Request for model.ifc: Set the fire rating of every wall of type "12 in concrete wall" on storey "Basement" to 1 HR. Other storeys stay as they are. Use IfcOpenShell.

First a look at what the model holds.

```python
import ifcopenshell
import ifcopenshell.util.element

model = ifcopenshell.open("model.ifc")
print(model.schema)
storey = next(s for s in model.by_type("IfcBuildingStorey") if s.Name == "Basement")
walls = [e for e in ifcopenshell.util.element.get_decomposition(storey) if e.is_a("IfcWall")]
seen = {}
for e in walls:
    element_type = ifcopenshell.util.element.get_type(e)
    key = (element_type.Name if element_type != e and element_type else None, ifcopenshell.util.element.get_pset(e, "Pset_WallCommon", "FireRating"))
    seen[key] = seen.get(key, 0) + 1
for (name, value), count in sorted(seen.items(), key=str):
    print(count, "x", name, "|", value)
```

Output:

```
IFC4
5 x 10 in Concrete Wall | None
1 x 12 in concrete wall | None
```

```python
import ifcopenshell
import ifcopenshell.api.pset
import ifcopenshell.util.element

model = ifcopenshell.open("model.ifc")

storey = next(s for s in model.by_type("IfcBuildingStorey") if s.Name == "Basement")
walls = [e for e in ifcopenshell.util.element.get_decomposition(storey) if e.is_a("IfcWall")]

count = 0
for e in walls:
    element_type = ifcopenshell.util.element.get_type(e)
    if element_type in (None, e) or element_type.Name != "12 in concrete wall":
        continue
    # add_pset returns the element's existing set when there is one.
    pset = ifcopenshell.api.pset.add_pset(model, product=e, name="Pset_WallCommon")
    ifcopenshell.api.pset.edit_pset(model, pset=pset, properties={"FireRating": "1 HR"})
    count += 1

print(count, "walls updated")

model.write("model_edited.ifc")
```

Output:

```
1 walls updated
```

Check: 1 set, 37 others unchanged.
